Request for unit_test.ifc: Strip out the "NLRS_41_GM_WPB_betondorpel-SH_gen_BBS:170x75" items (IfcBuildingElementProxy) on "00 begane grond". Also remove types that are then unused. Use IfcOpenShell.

First a look at what the model holds.

```python
import ifcopenshell
import ifcopenshell.util.element

model = ifcopenshell.open("unit_test.ifc")
print(model.schema)
storey = next(s for s in model.by_type("IfcBuildingStorey") if s.Name == "00 begane grond")
proxies = [e for e in ifcopenshell.util.element.get_decomposition(storey) if e.is_a("IfcBuildingElementProxy")]
seen = {}
for e in proxies:
    element_type = ifcopenshell.util.element.get_type(e)
    name = element_type.Name if element_type not in (None, e) else None
    seen[name] = seen.get(name, 0) + 1
for name, count in sorted(seen.items(), key=str):
    print(count, "x", name)
```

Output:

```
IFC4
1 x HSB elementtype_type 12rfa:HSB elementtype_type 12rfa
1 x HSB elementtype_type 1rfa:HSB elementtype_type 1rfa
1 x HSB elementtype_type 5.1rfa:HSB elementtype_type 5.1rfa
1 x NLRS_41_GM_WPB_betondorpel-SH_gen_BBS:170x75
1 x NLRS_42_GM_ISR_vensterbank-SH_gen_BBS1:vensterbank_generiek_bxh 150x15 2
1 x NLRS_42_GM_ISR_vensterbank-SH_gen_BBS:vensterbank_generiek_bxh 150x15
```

```python
import ifcopenshell
import ifcopenshell.api.root
import ifcopenshell.util.element

model = ifcopenshell.open("unit_test.ifc")

storey = next(s for s in model.by_type("IfcBuildingStorey") if s.Name == "00 begane grond")
proxies = [e for e in ifcopenshell.util.element.get_decomposition(storey) if e.is_a("IfcBuildingElementProxy")]
targets = [e for e in proxies if (t := ifcopenshell.util.element.get_type(e)) not in (None, e) and t.Name == "NLRS_41_GM_WPB_betondorpel-SH_gen_BBS:170x75"]
types = {ifcopenshell.util.element.get_type(e) for e in targets} - {None, *targets}

for e in targets:
    ifcopenshell.api.root.remove_product(model, product=e)
print(len(targets), "removed")

unused = [t for t in types if not ifcopenshell.util.element.get_types(t)]
for t in unused:
    ifcopenshell.api.root.remove_product(model, product=t)
print(len(unused), "unused types removed")

model.write("unit_test_v2.ifc")
```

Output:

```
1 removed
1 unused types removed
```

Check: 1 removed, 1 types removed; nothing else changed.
